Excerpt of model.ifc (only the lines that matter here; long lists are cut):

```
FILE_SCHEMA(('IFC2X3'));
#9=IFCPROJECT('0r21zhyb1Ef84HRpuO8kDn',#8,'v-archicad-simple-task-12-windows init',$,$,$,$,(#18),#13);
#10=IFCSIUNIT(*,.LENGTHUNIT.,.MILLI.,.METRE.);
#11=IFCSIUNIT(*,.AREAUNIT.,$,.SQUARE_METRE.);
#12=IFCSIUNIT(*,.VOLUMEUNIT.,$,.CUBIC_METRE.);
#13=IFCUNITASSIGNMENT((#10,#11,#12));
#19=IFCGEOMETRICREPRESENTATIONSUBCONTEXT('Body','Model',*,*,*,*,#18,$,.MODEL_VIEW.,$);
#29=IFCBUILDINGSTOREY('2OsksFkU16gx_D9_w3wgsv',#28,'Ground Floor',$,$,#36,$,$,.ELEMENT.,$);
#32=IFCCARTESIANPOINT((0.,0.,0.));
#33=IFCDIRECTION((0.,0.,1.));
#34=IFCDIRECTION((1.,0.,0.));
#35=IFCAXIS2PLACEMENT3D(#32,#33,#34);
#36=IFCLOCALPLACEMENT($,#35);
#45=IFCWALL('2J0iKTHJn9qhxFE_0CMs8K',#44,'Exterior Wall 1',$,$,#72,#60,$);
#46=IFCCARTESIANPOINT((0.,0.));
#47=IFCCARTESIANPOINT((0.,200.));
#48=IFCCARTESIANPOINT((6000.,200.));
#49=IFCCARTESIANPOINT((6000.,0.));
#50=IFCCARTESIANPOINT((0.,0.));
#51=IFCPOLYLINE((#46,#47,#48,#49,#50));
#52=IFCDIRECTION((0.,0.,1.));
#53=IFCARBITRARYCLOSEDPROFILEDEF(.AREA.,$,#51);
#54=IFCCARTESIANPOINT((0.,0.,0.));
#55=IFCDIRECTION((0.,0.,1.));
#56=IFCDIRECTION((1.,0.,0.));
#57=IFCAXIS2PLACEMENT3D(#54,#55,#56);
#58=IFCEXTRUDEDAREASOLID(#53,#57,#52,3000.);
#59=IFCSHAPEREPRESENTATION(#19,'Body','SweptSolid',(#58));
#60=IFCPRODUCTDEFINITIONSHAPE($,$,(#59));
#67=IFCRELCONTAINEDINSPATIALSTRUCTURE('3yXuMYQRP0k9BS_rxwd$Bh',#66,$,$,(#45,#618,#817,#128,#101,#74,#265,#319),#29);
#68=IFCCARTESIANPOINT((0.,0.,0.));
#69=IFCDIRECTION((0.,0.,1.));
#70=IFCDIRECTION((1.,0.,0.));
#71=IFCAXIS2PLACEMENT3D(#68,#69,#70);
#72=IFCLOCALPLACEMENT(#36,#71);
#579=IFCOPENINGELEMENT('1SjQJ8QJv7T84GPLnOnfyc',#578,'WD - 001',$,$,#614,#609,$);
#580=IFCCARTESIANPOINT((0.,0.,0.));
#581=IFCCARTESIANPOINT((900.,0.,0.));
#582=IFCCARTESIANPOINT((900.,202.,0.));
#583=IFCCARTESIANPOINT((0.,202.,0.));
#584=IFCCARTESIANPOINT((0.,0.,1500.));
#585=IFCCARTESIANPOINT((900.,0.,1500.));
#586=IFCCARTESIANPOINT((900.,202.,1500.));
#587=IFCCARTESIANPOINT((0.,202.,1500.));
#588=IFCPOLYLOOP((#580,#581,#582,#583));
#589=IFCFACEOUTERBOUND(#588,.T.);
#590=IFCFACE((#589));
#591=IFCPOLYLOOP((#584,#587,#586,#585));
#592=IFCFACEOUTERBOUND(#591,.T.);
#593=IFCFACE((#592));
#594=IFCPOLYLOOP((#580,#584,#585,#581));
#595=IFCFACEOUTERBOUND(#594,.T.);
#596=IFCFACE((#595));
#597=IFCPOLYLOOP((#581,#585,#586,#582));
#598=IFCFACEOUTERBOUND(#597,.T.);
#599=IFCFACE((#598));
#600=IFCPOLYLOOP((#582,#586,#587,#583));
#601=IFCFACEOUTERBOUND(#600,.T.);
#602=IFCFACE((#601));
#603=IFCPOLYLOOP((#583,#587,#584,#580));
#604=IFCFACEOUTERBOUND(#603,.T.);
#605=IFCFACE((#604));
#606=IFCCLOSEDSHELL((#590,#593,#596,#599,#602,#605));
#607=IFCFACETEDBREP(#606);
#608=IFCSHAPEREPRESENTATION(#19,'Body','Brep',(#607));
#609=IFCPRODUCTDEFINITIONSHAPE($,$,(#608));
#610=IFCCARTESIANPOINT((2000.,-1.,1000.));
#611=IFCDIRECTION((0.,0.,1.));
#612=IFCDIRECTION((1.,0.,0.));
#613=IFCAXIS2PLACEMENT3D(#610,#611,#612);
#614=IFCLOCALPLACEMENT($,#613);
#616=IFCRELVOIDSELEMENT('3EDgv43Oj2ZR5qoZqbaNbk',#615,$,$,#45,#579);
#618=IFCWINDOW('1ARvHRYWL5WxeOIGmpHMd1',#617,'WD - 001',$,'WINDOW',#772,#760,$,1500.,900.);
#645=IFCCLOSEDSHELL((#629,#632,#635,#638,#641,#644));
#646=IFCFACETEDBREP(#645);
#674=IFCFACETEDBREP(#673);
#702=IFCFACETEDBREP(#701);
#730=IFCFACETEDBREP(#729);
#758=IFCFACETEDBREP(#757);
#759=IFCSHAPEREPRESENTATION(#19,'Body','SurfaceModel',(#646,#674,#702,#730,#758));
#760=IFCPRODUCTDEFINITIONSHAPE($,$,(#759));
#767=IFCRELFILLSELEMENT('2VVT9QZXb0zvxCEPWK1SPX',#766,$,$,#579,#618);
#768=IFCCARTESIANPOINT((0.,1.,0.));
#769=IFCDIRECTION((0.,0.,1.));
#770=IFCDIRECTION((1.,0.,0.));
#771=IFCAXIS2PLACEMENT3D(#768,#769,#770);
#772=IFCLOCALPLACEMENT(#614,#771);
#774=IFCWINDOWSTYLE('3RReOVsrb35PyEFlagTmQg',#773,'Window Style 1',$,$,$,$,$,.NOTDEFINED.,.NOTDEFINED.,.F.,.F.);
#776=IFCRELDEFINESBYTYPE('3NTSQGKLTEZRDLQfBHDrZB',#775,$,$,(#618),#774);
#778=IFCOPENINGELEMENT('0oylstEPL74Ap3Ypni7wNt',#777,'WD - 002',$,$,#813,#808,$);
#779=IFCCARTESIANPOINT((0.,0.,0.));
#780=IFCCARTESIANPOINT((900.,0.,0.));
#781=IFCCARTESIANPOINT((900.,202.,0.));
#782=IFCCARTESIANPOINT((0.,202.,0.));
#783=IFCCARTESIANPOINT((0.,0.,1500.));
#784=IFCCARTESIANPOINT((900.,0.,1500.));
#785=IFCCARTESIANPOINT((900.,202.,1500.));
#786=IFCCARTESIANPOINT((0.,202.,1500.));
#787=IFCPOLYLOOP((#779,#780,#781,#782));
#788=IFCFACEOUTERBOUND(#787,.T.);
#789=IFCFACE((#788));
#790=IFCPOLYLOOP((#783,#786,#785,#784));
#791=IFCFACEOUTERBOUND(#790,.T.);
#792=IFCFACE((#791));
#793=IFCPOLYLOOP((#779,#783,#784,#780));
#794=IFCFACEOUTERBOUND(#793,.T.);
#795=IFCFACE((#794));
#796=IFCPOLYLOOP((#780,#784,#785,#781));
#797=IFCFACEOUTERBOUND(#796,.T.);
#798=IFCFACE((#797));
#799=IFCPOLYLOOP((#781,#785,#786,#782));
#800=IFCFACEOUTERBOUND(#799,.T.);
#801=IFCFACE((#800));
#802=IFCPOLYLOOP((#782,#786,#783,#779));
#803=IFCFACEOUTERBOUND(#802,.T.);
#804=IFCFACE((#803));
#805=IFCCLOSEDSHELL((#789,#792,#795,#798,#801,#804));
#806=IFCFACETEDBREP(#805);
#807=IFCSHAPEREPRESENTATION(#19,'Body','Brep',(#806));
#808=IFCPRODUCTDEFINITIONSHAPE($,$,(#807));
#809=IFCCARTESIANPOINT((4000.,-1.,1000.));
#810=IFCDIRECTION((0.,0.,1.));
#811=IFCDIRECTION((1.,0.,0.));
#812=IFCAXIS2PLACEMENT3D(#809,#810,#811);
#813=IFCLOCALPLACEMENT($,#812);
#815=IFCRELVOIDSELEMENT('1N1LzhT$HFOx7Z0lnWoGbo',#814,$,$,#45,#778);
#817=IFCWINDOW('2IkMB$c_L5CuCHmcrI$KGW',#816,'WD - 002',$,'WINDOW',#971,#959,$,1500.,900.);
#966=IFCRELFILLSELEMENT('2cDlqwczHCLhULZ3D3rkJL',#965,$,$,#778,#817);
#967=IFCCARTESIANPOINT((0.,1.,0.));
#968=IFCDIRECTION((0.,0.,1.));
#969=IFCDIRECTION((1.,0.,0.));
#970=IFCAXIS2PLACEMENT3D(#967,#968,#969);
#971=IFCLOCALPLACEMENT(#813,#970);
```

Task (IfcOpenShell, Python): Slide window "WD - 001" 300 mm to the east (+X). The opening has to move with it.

```python
import ifcopenshell
import ifcopenshell.api.geometry
import ifcopenshell.util.placement

model = ifcopenshell.open("model.ifc")

window = model.by_guid("1ARvHRYWL5WxeOIGmpHMd1")
opening = window.FillsVoids[0].RelatingOpeningElement
wall = opening.VoidsElements[0].RelatingBuildingElement

wall_matrix = ifcopenshell.util.placement.get_local_placement(wall.ObjectPlacement)
shift = wall_matrix[:3, 0] * 300.0
before = ifcopenshell.util.placement.get_local_placement(window.ObjectPlacement)[:3, 3].copy()

# The window is placed relative to its opening, so it follows when the opening moves.
matrix = ifcopenshell.util.placement.get_local_placement(opening.ObjectPlacement)
matrix[:3, 3] += shift
ifcopenshell.api.geometry.edit_object_placement(
    model, product=opening, matrix=matrix, is_si=False, should_transform_children=True
)

after = ifcopenshell.util.placement.get_local_placement(window.ObjectPlacement)[:3, 3]
print("window moved by", (after - before).round(3) + 0.0)

model.write("model_updated.ifc")
```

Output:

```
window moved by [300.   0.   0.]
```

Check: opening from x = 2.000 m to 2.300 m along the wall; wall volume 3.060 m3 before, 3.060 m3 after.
